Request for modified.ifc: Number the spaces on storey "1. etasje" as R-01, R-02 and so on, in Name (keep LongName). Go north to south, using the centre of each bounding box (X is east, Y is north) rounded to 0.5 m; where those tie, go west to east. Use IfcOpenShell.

First a look at what the model holds.

```python
import ifcopenshell
import ifcopenshell.util.element
import ifcopenshell.util.placement

model = ifcopenshell.open("modified.ifc")
print(model.schema)
storey = next(s for s in model.by_type("IfcBuildingStorey") if s.Name == "1. etasje")
spaces = [e for e in ifcopenshell.util.element.get_decomposition(storey) if e.is_a("IfcSpace")]
for e in sorted(spaces, key=lambda e: e.id()):
    origin = ifcopenshell.util.placement.get_local_placement(e.ObjectPlacement)[:3, 3]
    print(e.id(), e.Name, e.LongName, origin.round(2) + 0.0, sep=" | ")
```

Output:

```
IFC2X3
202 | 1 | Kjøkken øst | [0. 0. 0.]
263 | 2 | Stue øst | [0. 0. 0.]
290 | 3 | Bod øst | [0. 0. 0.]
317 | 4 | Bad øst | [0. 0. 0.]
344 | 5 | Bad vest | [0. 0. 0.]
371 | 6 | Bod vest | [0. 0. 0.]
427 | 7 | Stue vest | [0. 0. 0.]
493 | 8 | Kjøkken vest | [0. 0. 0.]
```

```python
import ifcopenshell
import ifcopenshell.geom
import ifcopenshell.util.element
import ifcopenshell.util.shape

model = ifcopenshell.open("modified.ifc")
settings = ifcopenshell.geom.settings()
settings.set("use-world-coords", True)


def centre(element):
    shape = ifcopenshell.geom.create_shape(settings, element)
    return ifcopenshell.util.shape.get_bbox_centroid(shape.geometry)


storey = next(s for s in model.by_type("IfcBuildingStorey") if s.Name == "1. etasje")
spaces = [e for e in ifcopenshell.util.element.get_decomposition(storey) if e.is_a("IfcSpace")]

# Insertion points can sit at a corner or the storey origin, so sort by the geometry (in metres).
centres = {e: centre(e) for e in spaces}
spaces.sort(key=lambda e: (-round(centres[e][1] / 0.5), centres[e][0]))

for i, e in enumerate(spaces, start=1):
    number = f"R-{i:02d}"
    e.Name = number
    print(e.id(), number)

model.write("modified_edited.ifc")
```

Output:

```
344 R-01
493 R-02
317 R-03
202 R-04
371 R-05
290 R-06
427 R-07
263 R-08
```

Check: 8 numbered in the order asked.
